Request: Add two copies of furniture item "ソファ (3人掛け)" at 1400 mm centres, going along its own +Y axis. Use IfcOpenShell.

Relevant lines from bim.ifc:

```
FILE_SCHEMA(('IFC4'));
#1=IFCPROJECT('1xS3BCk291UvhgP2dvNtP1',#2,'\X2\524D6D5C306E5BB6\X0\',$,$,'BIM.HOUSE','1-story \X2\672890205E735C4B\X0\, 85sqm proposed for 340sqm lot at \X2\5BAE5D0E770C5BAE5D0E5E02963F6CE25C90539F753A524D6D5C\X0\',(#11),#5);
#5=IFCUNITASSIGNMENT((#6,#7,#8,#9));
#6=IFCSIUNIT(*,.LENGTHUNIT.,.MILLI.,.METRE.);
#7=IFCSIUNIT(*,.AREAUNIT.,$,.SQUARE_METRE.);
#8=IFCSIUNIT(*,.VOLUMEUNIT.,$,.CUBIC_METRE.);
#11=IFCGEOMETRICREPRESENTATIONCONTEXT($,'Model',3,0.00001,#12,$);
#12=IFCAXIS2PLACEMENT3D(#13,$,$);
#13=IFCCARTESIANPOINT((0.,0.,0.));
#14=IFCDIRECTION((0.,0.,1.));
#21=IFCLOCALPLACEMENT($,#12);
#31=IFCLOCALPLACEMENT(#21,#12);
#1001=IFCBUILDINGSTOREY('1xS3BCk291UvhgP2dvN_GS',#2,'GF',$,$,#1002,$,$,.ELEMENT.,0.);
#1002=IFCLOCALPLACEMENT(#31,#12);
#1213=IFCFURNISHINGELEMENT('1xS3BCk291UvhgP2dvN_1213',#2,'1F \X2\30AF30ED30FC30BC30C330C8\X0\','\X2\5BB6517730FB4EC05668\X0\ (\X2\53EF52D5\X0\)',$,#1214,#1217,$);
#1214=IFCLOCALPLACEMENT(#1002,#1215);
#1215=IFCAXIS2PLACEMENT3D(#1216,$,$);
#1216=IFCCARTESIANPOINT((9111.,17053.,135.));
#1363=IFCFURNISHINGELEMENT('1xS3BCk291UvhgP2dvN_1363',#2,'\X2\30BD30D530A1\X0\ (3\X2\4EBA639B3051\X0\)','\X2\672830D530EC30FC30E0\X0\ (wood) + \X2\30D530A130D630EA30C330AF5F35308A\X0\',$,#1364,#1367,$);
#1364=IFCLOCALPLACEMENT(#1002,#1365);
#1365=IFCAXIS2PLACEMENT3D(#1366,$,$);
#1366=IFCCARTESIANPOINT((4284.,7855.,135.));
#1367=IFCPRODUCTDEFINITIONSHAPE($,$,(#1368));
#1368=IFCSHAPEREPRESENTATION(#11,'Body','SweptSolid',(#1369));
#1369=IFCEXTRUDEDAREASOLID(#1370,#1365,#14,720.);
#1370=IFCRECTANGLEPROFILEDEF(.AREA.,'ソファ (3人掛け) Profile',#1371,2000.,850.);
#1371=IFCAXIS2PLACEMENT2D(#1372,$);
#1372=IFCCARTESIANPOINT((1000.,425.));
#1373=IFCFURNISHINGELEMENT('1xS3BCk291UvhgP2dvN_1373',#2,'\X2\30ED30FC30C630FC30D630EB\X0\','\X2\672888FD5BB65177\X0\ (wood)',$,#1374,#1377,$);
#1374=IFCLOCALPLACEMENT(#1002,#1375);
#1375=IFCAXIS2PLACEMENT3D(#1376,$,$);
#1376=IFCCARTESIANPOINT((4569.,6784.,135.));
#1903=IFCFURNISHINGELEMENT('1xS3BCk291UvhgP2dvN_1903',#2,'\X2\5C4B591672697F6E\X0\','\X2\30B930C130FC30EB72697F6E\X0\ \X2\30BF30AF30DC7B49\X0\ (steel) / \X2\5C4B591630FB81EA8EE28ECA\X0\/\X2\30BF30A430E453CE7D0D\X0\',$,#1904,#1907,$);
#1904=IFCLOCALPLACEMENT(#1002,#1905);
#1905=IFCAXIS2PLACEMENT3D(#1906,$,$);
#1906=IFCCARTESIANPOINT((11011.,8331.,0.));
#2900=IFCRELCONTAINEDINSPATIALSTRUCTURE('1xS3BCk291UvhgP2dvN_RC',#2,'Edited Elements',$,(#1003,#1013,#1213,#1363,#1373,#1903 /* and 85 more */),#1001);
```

```python
import ifcopenshell
import ifcopenshell.api.geometry
import ifcopenshell.api.root
import ifcopenshell.util.element
import ifcopenshell.util.placement
import ifcopenshell.util.unit

model = ifcopenshell.open("bim.ifc")
unit_scale = ifcopenshell.util.unit.calculate_unit_scale(model)


def reuse_history(source, copy):
    """copy_class also copies each property set's owner history, people and application; keep the originals."""
    for rel in copy.IsDefinedBy:
        if rel.is_a("IfcRelDefinesByProperties") and (history := rel.RelatingPropertyDefinition.OwnerHistory):
            rel.RelatingPropertyDefinition.OwnerHistory = source.OwnerHistory
            ifcopenshell.util.element.remove_deep2(model, history)


source = model.by_id(1363)
base = ifcopenshell.util.placement.get_local_placement(source.ObjectPlacement)
step = base[:3, 1] * 1.4 / unit_scale

for i in range(1, 3):
    copy = ifcopenshell.api.root.copy_class(model, product=source)
    copy.Representation = ifcopenshell.util.element.copy_deep(
        model, source.Representation, exclude=["IfcGeometricRepresentationContext", "IfcRepresentationMap"]
    )
    reuse_history(source, copy)
    matrix = base.copy()
    matrix[:3, 3] += i * step
    print("added at", matrix[:3, 3].round(3) + 0.0)
    ifcopenshell.api.geometry.edit_object_placement(model, product=copy, matrix=matrix, is_si=False)

model.write("bim_updated.ifc")
```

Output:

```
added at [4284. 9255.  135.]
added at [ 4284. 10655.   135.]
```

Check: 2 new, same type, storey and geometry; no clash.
